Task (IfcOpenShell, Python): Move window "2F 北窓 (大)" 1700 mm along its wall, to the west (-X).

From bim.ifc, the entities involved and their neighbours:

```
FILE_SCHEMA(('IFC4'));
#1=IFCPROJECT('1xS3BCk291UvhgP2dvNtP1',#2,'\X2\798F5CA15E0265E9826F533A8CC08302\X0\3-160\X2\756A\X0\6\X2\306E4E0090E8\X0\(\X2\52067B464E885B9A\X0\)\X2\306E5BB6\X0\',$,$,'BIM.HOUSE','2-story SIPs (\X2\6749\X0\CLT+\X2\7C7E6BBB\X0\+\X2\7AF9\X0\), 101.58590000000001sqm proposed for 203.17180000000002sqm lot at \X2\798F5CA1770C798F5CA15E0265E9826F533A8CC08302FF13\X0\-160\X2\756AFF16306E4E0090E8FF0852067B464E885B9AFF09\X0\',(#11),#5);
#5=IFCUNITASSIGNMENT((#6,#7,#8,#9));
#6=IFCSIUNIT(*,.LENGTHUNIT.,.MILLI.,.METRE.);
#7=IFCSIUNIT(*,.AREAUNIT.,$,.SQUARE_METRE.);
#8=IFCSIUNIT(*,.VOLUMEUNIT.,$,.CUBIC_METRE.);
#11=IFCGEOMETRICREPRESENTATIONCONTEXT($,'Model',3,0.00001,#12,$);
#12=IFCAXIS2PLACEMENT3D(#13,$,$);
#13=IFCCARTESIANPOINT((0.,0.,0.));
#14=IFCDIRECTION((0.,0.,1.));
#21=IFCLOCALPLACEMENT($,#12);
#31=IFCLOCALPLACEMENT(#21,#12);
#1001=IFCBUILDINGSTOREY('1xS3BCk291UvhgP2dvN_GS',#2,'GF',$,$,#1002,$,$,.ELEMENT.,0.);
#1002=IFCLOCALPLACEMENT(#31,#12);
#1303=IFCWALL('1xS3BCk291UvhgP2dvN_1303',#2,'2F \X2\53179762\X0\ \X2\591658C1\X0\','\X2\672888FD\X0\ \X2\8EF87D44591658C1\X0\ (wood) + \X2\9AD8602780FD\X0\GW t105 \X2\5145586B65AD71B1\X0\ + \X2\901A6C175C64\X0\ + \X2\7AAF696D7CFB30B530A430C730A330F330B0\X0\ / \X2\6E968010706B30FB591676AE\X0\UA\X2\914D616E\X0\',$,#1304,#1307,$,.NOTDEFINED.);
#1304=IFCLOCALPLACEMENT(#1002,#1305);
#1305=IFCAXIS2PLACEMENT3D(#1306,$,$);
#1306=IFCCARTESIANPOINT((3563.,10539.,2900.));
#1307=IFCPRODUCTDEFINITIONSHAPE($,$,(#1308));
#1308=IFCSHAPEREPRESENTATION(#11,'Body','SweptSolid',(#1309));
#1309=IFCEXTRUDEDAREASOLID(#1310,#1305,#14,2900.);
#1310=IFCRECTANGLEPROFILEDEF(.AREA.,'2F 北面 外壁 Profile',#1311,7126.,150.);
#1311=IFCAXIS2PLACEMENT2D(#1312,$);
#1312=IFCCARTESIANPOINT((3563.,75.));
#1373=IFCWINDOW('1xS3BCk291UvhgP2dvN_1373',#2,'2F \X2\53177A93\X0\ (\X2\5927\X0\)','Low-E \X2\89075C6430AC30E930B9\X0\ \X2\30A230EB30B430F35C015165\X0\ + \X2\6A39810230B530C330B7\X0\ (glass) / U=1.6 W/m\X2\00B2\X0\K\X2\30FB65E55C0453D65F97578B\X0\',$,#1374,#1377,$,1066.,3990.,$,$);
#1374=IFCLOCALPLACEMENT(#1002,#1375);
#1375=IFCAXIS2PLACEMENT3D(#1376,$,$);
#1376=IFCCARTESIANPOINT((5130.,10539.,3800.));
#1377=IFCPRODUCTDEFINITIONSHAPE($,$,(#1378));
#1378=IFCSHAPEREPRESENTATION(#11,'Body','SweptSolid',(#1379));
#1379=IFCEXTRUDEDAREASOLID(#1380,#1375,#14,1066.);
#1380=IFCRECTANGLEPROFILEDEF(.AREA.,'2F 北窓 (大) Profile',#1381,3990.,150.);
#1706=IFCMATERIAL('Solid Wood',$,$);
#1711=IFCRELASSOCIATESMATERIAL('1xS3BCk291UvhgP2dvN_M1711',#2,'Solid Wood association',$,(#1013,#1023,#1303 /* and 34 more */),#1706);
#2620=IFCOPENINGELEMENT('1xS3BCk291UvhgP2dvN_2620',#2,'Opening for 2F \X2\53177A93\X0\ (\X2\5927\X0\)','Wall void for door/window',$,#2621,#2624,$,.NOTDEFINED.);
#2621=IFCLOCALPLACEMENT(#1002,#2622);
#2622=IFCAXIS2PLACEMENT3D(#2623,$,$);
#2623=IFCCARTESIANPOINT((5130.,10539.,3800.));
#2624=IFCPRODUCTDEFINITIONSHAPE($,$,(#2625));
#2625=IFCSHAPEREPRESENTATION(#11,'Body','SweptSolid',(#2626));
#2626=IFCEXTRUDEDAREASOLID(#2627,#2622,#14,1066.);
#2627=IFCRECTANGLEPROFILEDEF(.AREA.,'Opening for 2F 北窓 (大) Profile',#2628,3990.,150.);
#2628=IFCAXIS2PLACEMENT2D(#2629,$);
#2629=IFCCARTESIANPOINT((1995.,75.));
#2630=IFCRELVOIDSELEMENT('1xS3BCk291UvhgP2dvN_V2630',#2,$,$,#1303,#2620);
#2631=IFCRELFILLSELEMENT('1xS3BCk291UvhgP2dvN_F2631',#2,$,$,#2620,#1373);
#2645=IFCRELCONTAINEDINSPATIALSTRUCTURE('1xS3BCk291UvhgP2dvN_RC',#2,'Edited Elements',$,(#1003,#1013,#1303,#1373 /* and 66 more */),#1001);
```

```python
import ifcopenshell
import ifcopenshell.api.geometry
import ifcopenshell.util.placement
import ifcopenshell.util.unit

model = ifcopenshell.open("bim.ifc")
unit_scale = ifcopenshell.util.unit.calculate_unit_scale(model)

window = model.by_guid("1xS3BCk291UvhgP2dvN_1373")
opening = window.FillsVoids[0].RelatingOpeningElement
wall = opening.VoidsElements[0].RelatingBuildingElement

wall_matrix = ifcopenshell.util.placement.get_local_placement(wall.ObjectPlacement)
shift = wall_matrix[:3, 0] * -1.7 / unit_scale
before = ifcopenshell.util.placement.get_local_placement(window.ObjectPlacement)[:3, 3].copy()

# The window is not placed relative to its opening, so move both.
for product in (opening, window):
    matrix = ifcopenshell.util.placement.get_local_placement(product.ObjectPlacement)
    matrix[:3, 3] += shift
    ifcopenshell.api.geometry.edit_object_placement(model, product=product, matrix=matrix, is_si=False)

after = ifcopenshell.util.placement.get_local_placement(window.ObjectPlacement)[:3, 3]
print("window moved by", (after - before).round(3) + 0.0)

model.write("bim-out.ifc")
```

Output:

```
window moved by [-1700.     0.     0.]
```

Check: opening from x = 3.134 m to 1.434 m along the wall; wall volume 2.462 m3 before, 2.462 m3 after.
